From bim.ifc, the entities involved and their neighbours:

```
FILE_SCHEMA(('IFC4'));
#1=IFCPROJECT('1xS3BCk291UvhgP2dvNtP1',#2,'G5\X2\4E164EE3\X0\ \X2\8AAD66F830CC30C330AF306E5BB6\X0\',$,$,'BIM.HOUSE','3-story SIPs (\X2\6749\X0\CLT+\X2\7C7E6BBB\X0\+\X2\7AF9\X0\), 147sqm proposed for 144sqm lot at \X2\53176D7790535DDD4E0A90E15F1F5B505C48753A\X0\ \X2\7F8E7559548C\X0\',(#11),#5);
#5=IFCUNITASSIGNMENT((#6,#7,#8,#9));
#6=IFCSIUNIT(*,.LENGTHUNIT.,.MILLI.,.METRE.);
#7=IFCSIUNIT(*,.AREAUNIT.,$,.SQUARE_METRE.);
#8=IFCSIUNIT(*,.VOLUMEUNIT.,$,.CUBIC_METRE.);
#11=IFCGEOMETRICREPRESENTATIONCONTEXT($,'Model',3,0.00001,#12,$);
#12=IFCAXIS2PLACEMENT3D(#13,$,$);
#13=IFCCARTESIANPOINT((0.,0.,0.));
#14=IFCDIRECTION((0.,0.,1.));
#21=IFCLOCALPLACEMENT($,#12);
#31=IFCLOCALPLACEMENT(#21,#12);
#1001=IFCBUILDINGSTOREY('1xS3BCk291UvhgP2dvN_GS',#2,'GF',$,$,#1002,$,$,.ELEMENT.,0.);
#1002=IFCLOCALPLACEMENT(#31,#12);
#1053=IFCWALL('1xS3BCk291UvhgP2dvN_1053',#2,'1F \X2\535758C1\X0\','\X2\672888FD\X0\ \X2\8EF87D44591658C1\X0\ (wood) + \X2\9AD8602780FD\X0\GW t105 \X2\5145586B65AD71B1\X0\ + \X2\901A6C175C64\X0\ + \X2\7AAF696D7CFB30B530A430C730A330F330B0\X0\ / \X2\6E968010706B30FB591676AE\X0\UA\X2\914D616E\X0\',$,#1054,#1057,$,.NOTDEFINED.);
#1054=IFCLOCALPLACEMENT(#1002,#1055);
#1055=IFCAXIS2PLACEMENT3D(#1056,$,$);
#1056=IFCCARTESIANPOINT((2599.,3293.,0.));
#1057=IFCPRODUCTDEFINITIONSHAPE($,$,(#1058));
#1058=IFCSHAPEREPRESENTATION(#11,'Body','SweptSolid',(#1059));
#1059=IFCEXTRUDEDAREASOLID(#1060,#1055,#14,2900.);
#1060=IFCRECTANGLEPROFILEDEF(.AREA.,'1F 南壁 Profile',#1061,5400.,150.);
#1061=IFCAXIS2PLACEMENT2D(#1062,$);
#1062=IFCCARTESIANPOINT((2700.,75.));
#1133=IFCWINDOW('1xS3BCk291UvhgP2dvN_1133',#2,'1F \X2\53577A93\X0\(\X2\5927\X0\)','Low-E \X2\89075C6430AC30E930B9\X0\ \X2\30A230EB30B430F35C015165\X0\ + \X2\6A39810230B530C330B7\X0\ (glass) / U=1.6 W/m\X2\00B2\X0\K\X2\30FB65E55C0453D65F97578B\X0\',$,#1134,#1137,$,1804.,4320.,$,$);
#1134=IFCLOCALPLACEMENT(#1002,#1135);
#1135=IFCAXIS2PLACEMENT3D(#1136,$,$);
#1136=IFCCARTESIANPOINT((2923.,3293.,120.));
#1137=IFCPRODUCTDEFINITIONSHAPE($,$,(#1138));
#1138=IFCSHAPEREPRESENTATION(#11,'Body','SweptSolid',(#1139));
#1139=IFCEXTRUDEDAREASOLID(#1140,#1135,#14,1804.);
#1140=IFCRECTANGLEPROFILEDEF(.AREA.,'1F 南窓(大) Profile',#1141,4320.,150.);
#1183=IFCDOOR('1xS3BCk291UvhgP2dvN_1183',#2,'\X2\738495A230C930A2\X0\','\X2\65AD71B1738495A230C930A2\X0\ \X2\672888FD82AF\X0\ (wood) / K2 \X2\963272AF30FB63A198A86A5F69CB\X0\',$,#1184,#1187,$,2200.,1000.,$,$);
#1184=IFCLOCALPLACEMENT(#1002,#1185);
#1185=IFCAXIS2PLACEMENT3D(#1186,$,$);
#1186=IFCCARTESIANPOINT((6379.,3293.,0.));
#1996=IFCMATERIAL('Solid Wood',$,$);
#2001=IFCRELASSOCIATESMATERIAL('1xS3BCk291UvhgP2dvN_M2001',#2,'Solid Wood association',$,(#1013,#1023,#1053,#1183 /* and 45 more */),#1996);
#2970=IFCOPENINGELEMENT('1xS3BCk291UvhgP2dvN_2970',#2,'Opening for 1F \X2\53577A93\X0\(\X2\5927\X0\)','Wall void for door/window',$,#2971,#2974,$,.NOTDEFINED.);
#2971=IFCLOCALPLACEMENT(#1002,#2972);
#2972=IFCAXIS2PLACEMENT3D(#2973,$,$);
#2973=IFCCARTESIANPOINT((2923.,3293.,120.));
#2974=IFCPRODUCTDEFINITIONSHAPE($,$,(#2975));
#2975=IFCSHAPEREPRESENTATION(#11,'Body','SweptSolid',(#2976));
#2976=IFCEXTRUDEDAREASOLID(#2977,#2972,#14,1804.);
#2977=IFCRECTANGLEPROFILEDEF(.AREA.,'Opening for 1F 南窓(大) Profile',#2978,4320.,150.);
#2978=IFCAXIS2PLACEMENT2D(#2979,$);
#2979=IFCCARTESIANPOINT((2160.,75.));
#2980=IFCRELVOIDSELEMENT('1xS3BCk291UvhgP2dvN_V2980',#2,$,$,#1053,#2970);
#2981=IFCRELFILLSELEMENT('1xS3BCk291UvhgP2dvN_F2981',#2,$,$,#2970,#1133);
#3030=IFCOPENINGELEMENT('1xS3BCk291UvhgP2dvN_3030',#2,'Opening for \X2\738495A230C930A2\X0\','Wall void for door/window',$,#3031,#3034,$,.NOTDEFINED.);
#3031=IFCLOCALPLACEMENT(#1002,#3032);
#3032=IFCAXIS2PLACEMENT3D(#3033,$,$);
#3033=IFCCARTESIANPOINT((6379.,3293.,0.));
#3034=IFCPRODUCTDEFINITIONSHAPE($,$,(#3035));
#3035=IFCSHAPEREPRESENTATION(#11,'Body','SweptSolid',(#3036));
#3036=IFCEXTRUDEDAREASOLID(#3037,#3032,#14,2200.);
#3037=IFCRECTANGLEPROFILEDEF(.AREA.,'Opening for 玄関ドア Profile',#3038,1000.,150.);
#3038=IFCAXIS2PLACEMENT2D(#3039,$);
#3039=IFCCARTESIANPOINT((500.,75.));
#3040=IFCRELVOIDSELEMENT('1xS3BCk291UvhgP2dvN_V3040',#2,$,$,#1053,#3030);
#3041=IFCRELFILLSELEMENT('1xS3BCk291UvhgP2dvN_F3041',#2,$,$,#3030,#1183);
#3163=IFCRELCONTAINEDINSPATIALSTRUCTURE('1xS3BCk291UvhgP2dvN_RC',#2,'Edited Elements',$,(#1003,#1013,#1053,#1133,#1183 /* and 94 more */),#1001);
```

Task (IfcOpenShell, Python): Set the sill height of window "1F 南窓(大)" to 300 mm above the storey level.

```python
import numpy as np
import ifcopenshell
import ifcopenshell.api.geometry
import ifcopenshell.geom
import ifcopenshell.util.element
import ifcopenshell.util.placement
import ifcopenshell.util.shape
import ifcopenshell.util.unit

model = ifcopenshell.open("bim.ifc")
unit_scale = ifcopenshell.util.unit.calculate_unit_scale(model)

window = model.by_id(1133)
opening = window.FillsVoids[0].RelatingOpeningElement
storey = ifcopenshell.util.element.get_container(window, ifc_class="IfcBuildingStorey")
level = ifcopenshell.util.placement.get_local_placement(storey.ObjectPlacement)[2, 3]

# The opening's origin need not be at the sill, so measure its lowest point.
shape = ifcopenshell.geom.create_shape(ifcopenshell.geom.settings(), opening)
bottom = ifcopenshell.util.shape.get_shape_bottom_elevation(shape, shape.geometry) / unit_scale
dz = level + 300.0 - bottom

shift = np.array([0.0, 0.0, dz])
# The window is not placed relative to its opening, so move both.
for product in (opening, window):
    matrix = ifcopenshell.util.placement.get_local_placement(product.ObjectPlacement)
    matrix[:3, 3] += shift
    ifcopenshell.api.geometry.edit_object_placement(model, product=product, matrix=matrix, is_si=False)

print(f"moved by {dz * unit_scale:+.3f} m")

model.write("bim_updated.ifc")
```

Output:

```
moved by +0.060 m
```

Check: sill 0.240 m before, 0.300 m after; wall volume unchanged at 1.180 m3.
